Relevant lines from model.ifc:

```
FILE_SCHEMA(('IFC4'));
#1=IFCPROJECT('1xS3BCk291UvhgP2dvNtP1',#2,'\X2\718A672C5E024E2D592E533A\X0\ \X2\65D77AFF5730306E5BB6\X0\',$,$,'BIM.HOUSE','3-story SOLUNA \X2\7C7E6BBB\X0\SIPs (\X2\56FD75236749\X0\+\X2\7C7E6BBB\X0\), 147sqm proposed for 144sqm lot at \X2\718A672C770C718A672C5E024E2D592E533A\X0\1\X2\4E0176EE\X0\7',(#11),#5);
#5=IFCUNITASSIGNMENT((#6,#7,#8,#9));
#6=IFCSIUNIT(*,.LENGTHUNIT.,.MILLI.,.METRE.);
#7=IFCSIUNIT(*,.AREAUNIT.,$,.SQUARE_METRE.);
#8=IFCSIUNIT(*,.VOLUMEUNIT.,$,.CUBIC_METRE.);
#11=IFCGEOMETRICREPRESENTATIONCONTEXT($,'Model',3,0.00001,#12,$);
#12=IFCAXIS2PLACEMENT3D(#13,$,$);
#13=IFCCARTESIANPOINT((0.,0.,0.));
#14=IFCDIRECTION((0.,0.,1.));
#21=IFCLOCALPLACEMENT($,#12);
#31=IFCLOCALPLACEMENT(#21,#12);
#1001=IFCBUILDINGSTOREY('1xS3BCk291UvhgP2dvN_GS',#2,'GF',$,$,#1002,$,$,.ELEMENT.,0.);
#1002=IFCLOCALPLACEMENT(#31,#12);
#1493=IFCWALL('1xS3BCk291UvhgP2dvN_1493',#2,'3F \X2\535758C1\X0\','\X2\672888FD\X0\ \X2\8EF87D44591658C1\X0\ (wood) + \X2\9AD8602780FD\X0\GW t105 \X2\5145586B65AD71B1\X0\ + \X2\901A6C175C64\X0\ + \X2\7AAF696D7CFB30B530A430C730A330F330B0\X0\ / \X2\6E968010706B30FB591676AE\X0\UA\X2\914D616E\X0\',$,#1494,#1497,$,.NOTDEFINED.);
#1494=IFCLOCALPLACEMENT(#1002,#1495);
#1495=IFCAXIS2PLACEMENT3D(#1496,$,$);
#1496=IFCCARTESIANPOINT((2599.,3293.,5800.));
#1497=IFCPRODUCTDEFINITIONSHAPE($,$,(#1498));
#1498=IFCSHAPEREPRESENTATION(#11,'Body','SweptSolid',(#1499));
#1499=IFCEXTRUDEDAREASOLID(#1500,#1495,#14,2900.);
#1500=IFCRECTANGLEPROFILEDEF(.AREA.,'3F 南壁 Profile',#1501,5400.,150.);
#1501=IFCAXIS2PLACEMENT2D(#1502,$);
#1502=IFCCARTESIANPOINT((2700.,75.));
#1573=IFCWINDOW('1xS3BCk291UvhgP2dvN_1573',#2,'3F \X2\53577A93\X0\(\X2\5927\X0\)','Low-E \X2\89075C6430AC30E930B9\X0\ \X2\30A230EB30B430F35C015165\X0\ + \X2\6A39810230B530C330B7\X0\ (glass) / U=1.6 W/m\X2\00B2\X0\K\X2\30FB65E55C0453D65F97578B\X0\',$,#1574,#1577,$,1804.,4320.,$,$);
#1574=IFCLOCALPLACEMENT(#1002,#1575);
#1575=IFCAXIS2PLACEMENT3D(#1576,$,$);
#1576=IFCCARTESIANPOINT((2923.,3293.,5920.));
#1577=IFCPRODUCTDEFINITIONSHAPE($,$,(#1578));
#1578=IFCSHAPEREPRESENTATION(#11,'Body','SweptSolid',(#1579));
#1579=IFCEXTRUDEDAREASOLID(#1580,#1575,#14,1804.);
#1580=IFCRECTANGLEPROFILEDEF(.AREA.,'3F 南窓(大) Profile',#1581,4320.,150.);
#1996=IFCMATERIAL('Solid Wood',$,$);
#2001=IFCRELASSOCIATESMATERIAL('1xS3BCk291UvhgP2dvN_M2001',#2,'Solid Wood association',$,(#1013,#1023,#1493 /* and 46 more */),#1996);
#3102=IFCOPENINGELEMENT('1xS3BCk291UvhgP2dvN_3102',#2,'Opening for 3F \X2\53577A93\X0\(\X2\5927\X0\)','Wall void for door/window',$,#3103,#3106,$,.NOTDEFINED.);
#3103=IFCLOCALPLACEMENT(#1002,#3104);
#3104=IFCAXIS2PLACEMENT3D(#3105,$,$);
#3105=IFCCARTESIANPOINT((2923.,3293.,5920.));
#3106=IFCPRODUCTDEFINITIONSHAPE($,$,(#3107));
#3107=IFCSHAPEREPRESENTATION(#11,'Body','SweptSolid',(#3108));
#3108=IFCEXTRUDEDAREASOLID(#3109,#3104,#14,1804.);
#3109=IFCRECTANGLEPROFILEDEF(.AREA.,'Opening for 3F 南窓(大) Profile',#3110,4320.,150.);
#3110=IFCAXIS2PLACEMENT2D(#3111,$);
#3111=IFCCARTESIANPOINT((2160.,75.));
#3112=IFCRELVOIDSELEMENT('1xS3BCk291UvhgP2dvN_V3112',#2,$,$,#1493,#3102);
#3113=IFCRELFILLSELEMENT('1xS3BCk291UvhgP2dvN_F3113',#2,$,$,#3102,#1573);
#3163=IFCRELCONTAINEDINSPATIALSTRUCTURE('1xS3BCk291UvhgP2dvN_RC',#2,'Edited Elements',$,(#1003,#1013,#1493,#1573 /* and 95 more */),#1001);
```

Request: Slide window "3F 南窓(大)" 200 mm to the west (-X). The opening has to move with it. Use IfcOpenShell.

```python
import ifcopenshell
import ifcopenshell.api.geometry
import ifcopenshell.util.placement
import ifcopenshell.util.unit

model = ifcopenshell.open("model.ifc")
unit_scale = ifcopenshell.util.unit.calculate_unit_scale(model)

window = model.by_id(1573)
opening = window.FillsVoids[0].RelatingOpeningElement
wall = opening.VoidsElements[0].RelatingBuildingElement

wall_matrix = ifcopenshell.util.placement.get_local_placement(wall.ObjectPlacement)
shift = wall_matrix[:3, 0] * -0.2 / unit_scale
before = ifcopenshell.util.placement.get_local_placement(window.ObjectPlacement)[:3, 3].copy()

# The window is not placed relative to its opening, so move both.
for product in (opening, window):
    matrix = ifcopenshell.util.placement.get_local_placement(product.ObjectPlacement)
    matrix[:3, 3] += shift
    ifcopenshell.api.geometry.edit_object_placement(model, product=product, matrix=matrix, is_si=False)

after = ifcopenshell.util.placement.get_local_placement(window.ObjectPlacement)[:3, 3]
print("window moved by", (after - before).round(3) + 0.0)

model.write("model_rev.ifc")
```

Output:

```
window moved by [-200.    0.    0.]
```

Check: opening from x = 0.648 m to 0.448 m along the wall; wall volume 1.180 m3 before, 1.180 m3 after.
